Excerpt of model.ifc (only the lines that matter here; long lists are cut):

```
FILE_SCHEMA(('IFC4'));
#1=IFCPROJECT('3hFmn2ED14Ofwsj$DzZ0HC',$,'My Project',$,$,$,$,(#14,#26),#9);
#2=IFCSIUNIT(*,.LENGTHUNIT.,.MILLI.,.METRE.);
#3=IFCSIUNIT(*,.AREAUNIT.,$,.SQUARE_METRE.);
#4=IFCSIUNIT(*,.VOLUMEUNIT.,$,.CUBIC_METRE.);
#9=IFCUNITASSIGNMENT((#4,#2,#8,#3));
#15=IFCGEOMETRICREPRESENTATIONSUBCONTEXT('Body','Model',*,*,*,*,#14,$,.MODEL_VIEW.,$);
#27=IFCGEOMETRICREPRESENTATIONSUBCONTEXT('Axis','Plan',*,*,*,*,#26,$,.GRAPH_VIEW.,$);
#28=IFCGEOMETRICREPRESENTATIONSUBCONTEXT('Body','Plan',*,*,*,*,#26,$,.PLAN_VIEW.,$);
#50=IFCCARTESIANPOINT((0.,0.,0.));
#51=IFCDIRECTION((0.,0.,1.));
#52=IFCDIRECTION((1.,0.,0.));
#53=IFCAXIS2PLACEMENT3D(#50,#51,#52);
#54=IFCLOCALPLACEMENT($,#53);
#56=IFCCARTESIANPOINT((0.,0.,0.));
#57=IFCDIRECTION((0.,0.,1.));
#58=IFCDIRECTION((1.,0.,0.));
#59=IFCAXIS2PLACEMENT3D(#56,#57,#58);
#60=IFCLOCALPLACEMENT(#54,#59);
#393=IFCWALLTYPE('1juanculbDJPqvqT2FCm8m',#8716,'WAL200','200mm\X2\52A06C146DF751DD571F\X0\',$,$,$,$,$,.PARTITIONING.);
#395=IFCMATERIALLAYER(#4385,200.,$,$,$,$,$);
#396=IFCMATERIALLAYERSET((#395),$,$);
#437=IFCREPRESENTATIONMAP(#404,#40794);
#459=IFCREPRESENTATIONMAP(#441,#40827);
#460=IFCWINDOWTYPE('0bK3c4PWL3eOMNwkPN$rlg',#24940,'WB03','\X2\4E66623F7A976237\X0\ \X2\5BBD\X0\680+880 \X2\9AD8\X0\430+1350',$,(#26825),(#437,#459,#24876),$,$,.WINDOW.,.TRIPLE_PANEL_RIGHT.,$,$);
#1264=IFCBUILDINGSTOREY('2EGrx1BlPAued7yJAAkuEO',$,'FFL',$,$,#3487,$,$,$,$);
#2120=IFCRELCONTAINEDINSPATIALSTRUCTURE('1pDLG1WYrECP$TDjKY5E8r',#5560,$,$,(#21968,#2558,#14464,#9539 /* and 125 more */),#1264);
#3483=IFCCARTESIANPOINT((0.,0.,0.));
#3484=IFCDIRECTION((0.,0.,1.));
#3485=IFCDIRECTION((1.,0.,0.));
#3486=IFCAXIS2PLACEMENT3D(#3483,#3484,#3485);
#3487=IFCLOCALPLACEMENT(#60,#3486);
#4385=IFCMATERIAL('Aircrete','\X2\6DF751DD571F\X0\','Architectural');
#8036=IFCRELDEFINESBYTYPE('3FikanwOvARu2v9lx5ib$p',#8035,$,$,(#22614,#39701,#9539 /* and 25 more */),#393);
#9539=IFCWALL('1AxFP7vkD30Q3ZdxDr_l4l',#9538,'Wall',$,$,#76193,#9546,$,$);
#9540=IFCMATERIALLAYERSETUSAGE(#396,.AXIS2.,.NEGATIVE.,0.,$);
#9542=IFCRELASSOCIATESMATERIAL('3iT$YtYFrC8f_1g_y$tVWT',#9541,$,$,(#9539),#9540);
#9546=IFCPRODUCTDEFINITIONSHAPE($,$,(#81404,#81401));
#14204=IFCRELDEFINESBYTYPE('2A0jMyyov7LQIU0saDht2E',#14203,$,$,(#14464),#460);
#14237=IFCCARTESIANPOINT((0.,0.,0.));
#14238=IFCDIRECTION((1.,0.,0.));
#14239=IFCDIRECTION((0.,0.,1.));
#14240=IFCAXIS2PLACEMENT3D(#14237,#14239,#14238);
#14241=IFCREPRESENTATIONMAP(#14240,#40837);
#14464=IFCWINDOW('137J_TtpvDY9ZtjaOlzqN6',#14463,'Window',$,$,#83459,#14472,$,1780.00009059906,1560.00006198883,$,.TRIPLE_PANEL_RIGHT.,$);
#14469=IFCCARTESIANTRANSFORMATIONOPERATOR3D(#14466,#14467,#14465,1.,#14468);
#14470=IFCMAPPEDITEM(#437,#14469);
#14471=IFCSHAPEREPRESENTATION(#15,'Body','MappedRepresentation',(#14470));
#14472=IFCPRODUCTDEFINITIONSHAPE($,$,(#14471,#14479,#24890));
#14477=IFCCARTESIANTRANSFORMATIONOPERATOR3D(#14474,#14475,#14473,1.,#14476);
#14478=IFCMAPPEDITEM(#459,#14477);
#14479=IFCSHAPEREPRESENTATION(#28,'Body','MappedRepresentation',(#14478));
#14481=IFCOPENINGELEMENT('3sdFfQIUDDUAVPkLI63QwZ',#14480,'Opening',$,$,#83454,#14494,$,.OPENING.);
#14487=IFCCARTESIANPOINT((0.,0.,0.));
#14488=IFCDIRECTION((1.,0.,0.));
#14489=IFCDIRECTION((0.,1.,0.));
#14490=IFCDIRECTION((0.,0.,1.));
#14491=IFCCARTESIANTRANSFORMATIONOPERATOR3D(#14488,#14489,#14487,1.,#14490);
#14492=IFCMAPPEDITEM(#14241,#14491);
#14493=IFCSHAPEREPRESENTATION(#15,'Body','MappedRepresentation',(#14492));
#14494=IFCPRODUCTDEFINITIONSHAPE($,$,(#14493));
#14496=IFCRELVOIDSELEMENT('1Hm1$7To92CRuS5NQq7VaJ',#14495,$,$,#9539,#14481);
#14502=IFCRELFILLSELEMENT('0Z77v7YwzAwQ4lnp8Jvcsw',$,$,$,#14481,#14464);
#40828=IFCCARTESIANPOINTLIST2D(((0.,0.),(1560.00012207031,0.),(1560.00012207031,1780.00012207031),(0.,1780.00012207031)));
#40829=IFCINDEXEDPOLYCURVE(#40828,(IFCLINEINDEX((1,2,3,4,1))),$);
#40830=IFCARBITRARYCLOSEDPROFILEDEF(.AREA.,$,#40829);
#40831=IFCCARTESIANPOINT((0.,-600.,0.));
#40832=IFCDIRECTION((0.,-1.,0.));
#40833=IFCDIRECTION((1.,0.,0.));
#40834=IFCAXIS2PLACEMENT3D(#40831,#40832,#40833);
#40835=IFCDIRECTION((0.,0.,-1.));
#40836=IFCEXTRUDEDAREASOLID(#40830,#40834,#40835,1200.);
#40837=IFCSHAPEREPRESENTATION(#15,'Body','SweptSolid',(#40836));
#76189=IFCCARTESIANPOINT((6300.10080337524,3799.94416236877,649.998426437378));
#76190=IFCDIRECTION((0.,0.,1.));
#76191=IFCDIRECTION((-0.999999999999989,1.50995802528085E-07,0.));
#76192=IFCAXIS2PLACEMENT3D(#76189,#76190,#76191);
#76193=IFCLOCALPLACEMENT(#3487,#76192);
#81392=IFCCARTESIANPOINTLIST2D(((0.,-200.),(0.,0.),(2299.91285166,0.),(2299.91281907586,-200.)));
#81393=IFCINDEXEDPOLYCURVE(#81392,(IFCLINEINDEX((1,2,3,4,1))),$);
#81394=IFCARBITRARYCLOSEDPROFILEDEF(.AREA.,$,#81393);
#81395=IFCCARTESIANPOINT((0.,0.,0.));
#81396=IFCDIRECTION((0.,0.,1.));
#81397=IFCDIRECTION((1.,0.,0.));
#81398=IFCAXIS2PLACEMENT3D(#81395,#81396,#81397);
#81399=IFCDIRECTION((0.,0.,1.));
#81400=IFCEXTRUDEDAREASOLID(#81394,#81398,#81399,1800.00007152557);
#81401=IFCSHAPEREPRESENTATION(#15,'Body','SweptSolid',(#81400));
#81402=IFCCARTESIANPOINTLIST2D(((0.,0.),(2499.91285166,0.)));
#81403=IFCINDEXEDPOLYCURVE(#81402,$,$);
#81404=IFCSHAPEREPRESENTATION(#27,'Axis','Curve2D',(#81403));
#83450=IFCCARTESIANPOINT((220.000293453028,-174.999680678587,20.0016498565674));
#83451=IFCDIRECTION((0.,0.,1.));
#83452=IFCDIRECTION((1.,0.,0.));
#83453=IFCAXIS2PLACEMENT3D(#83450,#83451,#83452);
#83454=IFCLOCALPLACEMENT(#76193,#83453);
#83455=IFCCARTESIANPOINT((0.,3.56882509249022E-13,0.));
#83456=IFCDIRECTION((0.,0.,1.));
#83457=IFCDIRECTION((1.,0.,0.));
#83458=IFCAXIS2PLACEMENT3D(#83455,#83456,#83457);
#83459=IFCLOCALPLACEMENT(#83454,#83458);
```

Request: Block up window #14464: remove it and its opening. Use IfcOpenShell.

```python
import ifcopenshell
import ifcopenshell.api.feature
import ifcopenshell.api.root
import ifcopenshell.geom
import ifcopenshell.util.shape

model = ifcopenshell.open("model.ifc")
settings = ifcopenshell.geom.settings()


def volume(element):
    """Net volume in cubic metres, openings subtracted."""
    shape = ifcopenshell.geom.create_shape(settings, element)
    return ifcopenshell.util.shape.get_volume(shape.geometry)


window = model.by_guid("137J_TtpvDY9ZtjaOlzqN6")
opening = window.FillsVoids[0].RelatingOpeningElement
wall = opening.VoidsElements[0].RelatingBuildingElement
before = volume(wall)

ifcopenshell.api.root.remove_product(model, product=window)
ifcopenshell.api.feature.remove_feature(model, feature=opening)

after = volume(wall)

print(f"wall volume {before:.3f} -> {after:.3f} m3")

model.write("model_updated.ifc")
```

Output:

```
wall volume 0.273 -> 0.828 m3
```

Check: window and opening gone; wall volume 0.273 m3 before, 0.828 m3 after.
